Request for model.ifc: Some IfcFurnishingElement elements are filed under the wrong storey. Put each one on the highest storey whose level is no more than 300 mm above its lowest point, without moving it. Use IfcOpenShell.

First a look at what the model holds.

```python
import ifcopenshell
import ifcopenshell.util.element
import ifcopenshell.util.placement

model = ifcopenshell.open("model.ifc")
print(model.schema)
for storey in model.by_type("IfcBuildingStorey"):
    level = ifcopenshell.util.placement.get_storey_elevation(storey)
    count = sum(e.is_a("IfcFurnishingElement") for e in ifcopenshell.util.element.get_contained(storey))
    print(storey.id(), storey.Name, round(level, 3), count, sep=" | ")
```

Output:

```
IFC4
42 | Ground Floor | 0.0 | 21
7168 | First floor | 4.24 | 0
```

```python
import ifcopenshell
import ifcopenshell.api.spatial
import ifcopenshell.geom
import ifcopenshell.util.element
import ifcopenshell.util.placement
import ifcopenshell.util.shape
import ifcopenshell.util.unit

model = ifcopenshell.open("model.ifc")
unit_scale = ifcopenshell.util.unit.calculate_unit_scale(model)
settings = ifcopenshell.geom.settings()

levels = sorted(
    ((ifcopenshell.util.placement.get_storey_elevation(s) * unit_scale, s) for s in model.by_type("IfcBuildingStorey")),
    key=lambda pair: pair[0],
)

for e in model.by_type("IfcFurnishingElement"):
    current = e.ContainedInStructure[0].RelatingStructure if e.ContainedInStructure else None
    if current is None or not current.is_a("IfcBuildingStorey"):
        continue
    shape = ifcopenshell.geom.create_shape(settings, e)
    bottom = ifcopenshell.util.shape.get_shape_bottom_elevation(shape, shape.geometry)
    below = [s for level, s in levels if level <= bottom + 0.3]
    storey = below[-1] if below else levels[0][1]
    if storey != current:
        # assign_container keeps the world position.
        ifcopenshell.api.spatial.assign_container(model, products=[e], relating_structure=storey)
        print(e.id(), current.Name, "->", storey.Name)

model.write("model_v2.ifc")
```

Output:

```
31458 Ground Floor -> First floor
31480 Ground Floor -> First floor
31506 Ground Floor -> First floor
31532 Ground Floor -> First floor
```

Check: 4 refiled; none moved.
